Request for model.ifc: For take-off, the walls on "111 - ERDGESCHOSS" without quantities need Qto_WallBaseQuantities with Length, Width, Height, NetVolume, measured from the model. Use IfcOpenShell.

First a look at what the model holds.

```python
import ifcopenshell
import ifcopenshell.util.element
import ifcopenshell.util.unit

model = ifcopenshell.open("model.ifc")
print(model.schema)
for unit_type in ("LENGTHUNIT", "AREAUNIT", "VOLUMEUNIT"):
    print(unit_type, ifcopenshell.util.unit.calculate_unit_scale(model, unit_type))
storey = next(s for s in model.by_type("IfcBuildingStorey") if s.Name == "111 - ERDGESCHOSS")
walls = [e for e in ifcopenshell.util.element.get_decomposition(storey) if e.is_a("IfcWall")]
for e in sorted(walls, key=lambda e: e.id()):
    print(e.id(), e.is_a(), e.Name, list(ifcopenshell.util.element.get_psets(e, qtos_only=True)), sep=" | ")
```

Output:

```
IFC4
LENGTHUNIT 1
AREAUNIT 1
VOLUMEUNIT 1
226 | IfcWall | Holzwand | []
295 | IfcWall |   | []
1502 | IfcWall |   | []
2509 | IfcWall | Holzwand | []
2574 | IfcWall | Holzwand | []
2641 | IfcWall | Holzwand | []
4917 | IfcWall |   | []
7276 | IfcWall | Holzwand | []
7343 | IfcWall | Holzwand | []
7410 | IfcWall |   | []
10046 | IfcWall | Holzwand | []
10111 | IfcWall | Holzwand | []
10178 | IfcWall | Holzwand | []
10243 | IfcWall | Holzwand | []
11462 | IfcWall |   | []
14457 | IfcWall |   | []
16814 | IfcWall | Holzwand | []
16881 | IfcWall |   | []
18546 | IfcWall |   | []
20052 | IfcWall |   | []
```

```python
import ifcopenshell
import ifcopenshell.api.pset
import ifcopenshell.geom
import ifcopenshell.util.element
import ifcopenshell.util.shape
import ifcopenshell.util.unit

model = ifcopenshell.open("model.ifc")
unit_scale = ifcopenshell.util.unit.calculate_unit_scale(model)
volume_scale = ifcopenshell.util.unit.calculate_unit_scale(model, "VOLUMEUNIT")
settings = ifcopenshell.geom.settings()

storey = next(s for s in model.by_type("IfcBuildingStorey") if s.Name == "111 - ERDGESCHOSS")
walls = [e for e in ifcopenshell.util.element.get_decomposition(storey) if e.is_a("IfcWall")]

for e in sorted(walls, key=lambda e: e.id()):
    if ifcopenshell.util.element.get_psets(e, qtos_only=True, should_inherit=False):
        continue
    # Geometry comes back in metres, in the element's own axes.
    shape = ifcopenshell.geom.create_shape(settings, e)
    values = {
        "Length": ifcopenshell.util.shape.get_x(shape.geometry) / unit_scale,
        "Width": ifcopenshell.util.shape.get_y(shape.geometry) / unit_scale,
        "Height": ifcopenshell.util.shape.get_z(shape.geometry) / unit_scale,
        "NetVolume": ifcopenshell.util.shape.get_volume(shape.geometry) / volume_scale,
    }
    qto = ifcopenshell.api.pset.add_qto(model, product=e, name="Qto_WallBaseQuantities")
    ifcopenshell.api.pset.edit_qto(model, qto=qto, properties=values)
    print(e.id(), {k: round(v, 3) for k, v in values.items()})

model.write("model_updated.ifc")
```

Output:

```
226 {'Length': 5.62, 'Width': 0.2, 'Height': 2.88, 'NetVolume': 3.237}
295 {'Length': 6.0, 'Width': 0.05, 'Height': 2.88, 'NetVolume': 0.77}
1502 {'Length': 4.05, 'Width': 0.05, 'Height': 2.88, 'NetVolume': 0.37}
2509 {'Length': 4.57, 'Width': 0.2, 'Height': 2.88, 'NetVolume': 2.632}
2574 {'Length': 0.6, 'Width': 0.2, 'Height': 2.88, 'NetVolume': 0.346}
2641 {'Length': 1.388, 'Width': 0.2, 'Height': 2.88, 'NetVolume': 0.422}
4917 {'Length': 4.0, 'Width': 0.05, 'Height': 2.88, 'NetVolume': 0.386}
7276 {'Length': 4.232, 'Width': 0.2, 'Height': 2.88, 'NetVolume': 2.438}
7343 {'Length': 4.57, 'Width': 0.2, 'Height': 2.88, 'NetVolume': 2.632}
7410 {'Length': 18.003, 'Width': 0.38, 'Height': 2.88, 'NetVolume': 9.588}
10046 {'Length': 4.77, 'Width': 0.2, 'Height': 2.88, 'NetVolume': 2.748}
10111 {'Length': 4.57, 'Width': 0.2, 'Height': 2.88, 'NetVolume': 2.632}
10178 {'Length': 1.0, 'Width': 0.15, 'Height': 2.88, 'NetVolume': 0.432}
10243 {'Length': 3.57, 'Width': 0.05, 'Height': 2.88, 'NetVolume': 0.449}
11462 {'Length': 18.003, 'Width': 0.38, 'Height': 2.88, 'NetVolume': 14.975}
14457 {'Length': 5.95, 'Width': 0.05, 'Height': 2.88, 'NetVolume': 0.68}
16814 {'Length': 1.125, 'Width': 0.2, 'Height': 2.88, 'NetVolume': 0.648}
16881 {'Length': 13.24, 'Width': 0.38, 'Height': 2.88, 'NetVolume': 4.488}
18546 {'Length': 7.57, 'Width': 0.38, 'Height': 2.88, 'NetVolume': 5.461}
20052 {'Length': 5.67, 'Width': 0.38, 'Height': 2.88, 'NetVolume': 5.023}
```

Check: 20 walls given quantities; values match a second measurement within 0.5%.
